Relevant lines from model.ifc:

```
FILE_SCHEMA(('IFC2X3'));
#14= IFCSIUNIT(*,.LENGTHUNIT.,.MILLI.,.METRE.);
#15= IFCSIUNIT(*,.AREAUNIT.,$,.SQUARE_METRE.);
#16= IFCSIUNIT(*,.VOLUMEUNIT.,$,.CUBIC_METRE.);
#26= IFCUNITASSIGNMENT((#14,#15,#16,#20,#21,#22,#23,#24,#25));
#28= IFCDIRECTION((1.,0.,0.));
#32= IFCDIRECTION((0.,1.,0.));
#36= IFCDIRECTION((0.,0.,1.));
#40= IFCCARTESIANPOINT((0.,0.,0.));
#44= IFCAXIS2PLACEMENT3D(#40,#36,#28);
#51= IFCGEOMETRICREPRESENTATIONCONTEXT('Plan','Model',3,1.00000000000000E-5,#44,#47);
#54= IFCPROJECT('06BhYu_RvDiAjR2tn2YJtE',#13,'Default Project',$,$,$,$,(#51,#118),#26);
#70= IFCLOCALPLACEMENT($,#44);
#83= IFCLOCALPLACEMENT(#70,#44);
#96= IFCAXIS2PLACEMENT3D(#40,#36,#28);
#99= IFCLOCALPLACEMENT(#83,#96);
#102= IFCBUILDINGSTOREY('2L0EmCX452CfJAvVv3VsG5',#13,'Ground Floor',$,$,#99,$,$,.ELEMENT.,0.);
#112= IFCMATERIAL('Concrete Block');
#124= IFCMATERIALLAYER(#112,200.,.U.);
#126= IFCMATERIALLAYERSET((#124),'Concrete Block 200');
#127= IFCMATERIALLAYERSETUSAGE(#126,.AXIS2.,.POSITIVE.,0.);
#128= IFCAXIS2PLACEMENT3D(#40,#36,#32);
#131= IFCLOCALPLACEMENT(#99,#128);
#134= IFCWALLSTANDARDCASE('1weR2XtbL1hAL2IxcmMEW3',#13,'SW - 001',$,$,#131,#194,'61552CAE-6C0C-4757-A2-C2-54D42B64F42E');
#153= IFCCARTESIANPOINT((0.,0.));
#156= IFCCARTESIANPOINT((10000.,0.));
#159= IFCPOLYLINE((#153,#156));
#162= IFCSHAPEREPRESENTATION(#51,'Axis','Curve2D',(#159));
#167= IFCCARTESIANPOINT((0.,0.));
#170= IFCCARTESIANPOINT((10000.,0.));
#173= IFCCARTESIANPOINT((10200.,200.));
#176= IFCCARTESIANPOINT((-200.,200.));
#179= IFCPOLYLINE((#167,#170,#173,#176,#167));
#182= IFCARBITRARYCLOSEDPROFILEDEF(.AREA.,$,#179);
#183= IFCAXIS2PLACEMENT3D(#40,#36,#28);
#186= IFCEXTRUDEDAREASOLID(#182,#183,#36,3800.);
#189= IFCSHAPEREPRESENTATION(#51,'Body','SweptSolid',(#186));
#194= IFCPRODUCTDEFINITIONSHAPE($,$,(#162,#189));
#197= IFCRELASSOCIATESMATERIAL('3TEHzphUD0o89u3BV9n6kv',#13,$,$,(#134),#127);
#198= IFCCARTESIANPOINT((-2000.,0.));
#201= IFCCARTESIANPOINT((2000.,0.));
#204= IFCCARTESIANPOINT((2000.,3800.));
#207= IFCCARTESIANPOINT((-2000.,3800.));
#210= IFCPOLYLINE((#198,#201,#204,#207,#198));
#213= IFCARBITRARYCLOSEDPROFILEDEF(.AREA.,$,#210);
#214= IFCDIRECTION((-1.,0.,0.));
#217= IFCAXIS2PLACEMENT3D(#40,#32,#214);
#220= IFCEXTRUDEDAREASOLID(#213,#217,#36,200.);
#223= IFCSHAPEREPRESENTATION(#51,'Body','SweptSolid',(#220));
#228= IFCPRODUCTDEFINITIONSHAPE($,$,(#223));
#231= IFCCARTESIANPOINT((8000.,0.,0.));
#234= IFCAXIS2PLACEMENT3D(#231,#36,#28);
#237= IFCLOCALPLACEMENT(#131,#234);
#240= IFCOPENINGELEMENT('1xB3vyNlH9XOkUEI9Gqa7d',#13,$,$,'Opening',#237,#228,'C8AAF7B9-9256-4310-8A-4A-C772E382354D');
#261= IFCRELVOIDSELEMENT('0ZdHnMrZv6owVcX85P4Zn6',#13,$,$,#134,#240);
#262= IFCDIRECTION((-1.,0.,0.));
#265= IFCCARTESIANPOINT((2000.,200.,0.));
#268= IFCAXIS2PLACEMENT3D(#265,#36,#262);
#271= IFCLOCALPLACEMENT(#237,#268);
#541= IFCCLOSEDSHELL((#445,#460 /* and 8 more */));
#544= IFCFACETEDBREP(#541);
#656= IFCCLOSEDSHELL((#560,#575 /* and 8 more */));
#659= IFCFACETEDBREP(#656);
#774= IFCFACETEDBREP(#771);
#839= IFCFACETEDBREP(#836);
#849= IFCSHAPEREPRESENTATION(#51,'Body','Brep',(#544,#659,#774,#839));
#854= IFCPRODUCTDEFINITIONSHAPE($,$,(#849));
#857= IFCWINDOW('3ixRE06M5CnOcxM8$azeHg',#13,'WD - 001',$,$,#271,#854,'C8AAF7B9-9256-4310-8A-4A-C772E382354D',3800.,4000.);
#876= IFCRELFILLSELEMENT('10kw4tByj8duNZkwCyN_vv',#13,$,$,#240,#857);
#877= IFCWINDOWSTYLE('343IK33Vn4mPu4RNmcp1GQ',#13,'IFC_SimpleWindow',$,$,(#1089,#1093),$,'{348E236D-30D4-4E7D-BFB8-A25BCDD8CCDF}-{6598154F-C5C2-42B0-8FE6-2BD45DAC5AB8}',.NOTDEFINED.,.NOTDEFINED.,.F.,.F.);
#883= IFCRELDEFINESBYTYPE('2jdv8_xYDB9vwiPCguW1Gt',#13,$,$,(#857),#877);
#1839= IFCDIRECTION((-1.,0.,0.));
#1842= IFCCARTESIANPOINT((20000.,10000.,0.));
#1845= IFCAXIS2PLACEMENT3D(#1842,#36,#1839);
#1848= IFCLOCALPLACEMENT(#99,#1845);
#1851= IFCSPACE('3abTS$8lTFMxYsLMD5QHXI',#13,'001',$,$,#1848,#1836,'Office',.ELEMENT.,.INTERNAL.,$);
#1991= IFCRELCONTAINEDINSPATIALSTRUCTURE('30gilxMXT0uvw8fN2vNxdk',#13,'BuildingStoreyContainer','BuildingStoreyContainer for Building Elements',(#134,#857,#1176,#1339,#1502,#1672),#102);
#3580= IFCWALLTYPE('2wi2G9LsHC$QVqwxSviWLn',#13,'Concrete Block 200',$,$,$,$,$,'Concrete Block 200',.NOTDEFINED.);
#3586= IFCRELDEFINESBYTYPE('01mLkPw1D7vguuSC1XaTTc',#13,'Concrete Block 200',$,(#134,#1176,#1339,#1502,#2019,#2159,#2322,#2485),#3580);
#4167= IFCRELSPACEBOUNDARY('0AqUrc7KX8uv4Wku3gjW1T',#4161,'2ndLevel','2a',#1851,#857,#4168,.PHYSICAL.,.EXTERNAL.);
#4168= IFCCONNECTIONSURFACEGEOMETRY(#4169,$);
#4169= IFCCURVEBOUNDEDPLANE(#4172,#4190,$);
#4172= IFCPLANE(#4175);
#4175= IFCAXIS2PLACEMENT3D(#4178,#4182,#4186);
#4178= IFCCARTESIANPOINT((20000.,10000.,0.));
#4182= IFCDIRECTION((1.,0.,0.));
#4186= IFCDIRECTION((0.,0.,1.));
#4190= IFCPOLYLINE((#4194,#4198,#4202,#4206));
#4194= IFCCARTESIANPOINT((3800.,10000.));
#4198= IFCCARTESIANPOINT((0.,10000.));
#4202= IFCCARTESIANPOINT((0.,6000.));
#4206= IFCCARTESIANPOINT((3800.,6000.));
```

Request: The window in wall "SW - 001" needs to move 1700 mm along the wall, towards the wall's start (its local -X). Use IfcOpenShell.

```python
import numpy as np
import ifcopenshell
import ifcopenshell.api.geometry
import ifcopenshell.util.placement

model = ifcopenshell.open("model.ifc")

window = model.by_guid("3ixRE06M5CnOcxM8$azeHg")
opening = window.FillsVoids[0].RelatingOpeningElement
wall = opening.VoidsElements[0].RelatingBuildingElement

wall_matrix = ifcopenshell.util.placement.get_local_placement(wall.ObjectPlacement)
shift = wall_matrix[:3, 0] * -1700.0
before = ifcopenshell.util.placement.get_local_placement(window.ObjectPlacement)[:3, 3].copy()

# The window is placed relative to its opening, so it follows when the opening moves.
matrix = ifcopenshell.util.placement.get_local_placement(opening.ObjectPlacement)
matrix[:3, 3] += shift
ifcopenshell.api.geometry.edit_object_placement(
    model, product=opening, matrix=matrix, is_si=False, should_transform_children=True
)

# Space boundary surfaces are stored in each space's coordinates; move them too.
for rel in window.ProvidesBoundaries:
    if not rel.ConnectionGeometry:
        continue
    surface = rel.ConnectionGeometry.SurfaceOnRelatingElement.BasisSurface
    space_matrix = ifcopenshell.util.placement.get_local_placement(rel.RelatingSpace.ObjectPlacement)
    point = np.array(surface.Position.Location.Coordinates) + space_matrix[:3, :3].T @ shift
    surface.Position = model.createIfcAxis2Placement3D(
        model.createIfcCartesianPoint(point.tolist()), surface.Position.Axis, surface.Position.RefDirection
    )

after = ifcopenshell.util.placement.get_local_placement(window.ObjectPlacement)[:3, 3]
print("window moved by", (after - before).round(3) + 0.0)

model.write("model_updated.ifc")
```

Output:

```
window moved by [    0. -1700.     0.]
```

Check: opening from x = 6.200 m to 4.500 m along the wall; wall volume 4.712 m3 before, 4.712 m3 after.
